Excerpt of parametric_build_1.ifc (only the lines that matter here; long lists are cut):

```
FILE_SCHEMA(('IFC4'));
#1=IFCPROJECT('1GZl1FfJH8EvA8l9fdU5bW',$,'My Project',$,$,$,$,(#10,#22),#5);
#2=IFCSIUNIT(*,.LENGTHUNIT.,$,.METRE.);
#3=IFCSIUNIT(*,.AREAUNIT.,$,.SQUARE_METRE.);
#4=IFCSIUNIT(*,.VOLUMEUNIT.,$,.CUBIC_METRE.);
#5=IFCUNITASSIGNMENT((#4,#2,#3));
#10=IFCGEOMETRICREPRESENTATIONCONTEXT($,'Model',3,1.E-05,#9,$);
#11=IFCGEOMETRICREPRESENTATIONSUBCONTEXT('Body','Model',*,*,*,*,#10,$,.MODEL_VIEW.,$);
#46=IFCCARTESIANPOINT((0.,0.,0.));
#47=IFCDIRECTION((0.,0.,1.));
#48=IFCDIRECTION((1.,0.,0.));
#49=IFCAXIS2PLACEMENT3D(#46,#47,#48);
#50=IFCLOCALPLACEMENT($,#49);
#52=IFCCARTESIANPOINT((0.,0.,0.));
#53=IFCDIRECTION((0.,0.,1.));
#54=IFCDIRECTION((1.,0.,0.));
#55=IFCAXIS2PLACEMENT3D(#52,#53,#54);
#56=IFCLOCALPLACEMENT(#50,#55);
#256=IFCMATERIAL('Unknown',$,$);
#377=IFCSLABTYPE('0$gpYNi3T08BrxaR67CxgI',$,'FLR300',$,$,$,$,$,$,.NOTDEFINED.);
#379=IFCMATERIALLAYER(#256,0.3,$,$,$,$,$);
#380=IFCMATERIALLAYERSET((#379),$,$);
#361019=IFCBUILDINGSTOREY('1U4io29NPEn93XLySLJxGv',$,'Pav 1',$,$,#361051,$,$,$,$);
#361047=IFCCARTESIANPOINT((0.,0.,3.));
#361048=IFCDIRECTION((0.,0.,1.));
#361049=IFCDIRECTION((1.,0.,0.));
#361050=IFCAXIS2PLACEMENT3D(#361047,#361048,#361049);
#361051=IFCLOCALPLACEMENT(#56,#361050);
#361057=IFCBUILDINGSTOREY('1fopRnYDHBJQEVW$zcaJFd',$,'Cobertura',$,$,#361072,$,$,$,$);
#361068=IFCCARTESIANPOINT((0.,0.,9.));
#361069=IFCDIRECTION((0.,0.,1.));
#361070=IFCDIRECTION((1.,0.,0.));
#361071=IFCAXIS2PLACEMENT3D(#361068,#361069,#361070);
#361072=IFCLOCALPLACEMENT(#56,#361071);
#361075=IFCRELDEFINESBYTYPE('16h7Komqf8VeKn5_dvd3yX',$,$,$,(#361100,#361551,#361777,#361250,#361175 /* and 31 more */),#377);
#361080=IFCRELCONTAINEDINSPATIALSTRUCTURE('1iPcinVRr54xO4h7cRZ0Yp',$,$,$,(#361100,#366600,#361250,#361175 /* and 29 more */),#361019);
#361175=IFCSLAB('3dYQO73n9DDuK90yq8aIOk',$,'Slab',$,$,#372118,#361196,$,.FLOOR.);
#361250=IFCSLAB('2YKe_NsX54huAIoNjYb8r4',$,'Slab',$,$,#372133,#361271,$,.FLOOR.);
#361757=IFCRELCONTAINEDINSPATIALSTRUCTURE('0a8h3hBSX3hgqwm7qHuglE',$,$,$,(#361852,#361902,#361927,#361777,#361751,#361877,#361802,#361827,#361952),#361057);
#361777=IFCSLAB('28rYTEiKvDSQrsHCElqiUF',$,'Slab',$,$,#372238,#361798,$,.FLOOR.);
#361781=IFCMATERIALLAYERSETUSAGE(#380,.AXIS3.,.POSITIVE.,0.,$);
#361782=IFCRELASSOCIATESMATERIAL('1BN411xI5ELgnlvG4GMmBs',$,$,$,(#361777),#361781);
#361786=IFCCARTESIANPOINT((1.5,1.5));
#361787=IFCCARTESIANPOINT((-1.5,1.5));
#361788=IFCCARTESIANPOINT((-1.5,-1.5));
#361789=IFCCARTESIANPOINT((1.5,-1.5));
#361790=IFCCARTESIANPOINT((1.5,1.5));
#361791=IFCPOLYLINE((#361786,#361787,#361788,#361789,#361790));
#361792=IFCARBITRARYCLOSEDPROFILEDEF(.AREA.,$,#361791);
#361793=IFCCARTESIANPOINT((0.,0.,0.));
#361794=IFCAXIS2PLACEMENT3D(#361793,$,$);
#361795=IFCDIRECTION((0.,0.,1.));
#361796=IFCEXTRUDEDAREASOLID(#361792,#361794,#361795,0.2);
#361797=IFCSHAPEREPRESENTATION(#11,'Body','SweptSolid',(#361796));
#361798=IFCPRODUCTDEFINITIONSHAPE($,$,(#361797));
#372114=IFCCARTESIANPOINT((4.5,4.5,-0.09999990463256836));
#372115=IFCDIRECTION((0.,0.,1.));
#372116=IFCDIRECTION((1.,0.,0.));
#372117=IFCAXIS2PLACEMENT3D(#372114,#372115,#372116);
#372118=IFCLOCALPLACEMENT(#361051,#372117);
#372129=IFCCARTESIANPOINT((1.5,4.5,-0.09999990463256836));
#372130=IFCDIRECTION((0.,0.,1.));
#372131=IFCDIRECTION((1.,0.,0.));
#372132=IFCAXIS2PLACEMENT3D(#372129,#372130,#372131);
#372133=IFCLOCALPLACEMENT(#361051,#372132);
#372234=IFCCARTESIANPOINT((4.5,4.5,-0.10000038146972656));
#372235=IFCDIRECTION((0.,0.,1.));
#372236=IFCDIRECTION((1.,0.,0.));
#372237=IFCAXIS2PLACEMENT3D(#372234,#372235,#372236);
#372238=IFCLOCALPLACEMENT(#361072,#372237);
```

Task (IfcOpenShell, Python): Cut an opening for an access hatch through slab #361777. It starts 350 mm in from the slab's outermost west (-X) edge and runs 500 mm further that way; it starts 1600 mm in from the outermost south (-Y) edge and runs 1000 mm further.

```python
import numpy as np
import ifcopenshell
import ifcopenshell.api.feature
import ifcopenshell.api.geometry
import ifcopenshell.api.root
import ifcopenshell.geom
import ifcopenshell.util.placement
import ifcopenshell.util.representation
import ifcopenshell.util.shape
import ifcopenshell.util.unit

model = ifcopenshell.open("parametric_build_1.ifc")
unit_scale = ifcopenshell.util.unit.calculate_unit_scale(model)
settings = ifcopenshell.geom.settings()


def volume(element):
    """Net volume in cubic metres, openings subtracted."""
    shape = ifcopenshell.geom.create_shape(settings, element)
    return ifcopenshell.util.shape.get_volume(shape.geometry)


slab = model.by_guid("28rYTEiKvDSQrsHCElqiUF")
before = volume(slab)

# Extent in the slab's own axes, in metres. The edges named are its -X and -Y sides.
slab_shape = ifcopenshell.geom.create_shape(settings, slab)
vertices = ifcopenshell.util.shape.get_vertices(slab_shape.geometry)
x_min, y_min, bottom = vertices.min(axis=0)
top = vertices[:, 2].max()

opening = ifcopenshell.api.root.create_entity(model, ifc_class="IfcOpeningElement", name="Access hatch opening", predefined_type="OPENING")
context = ifcopenshell.util.representation.get_context(model, "Model", "Body", "MODEL_VIEW")
width, depth = 0.5, 1
outline = [(0.0, 0.0), (width, 0.0), (width, depth), (0.0, depth), (0.0, 0.0)]
# Overshoot both faces by 50 mm so the cut is clean.
shape = ifcopenshell.api.geometry.add_slab_representation(
    model, context=context, depth=top - bottom + 0.1, polyline=outline
)
ifcopenshell.api.geometry.assign_representation(model, product=opening, representation=shape)

matrix = ifcopenshell.util.placement.get_local_placement(slab.ObjectPlacement)
matrix[:, 3] = matrix @ np.append(np.array([x_min + 0.35, y_min + 1.6, bottom - 0.05]) / unit_scale, 1.0)
ifcopenshell.api.geometry.edit_object_placement(model, product=opening, matrix=matrix, is_si=False)
ifcopenshell.api.feature.add_feature(model, feature=opening, element=slab)

after = volume(slab)

print(f"slab volume {before:.3f} -> {after:.3f} m3")

model.write("parametric_build_1_edited.ifc")
```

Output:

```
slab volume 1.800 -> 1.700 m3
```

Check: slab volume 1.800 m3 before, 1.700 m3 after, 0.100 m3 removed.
